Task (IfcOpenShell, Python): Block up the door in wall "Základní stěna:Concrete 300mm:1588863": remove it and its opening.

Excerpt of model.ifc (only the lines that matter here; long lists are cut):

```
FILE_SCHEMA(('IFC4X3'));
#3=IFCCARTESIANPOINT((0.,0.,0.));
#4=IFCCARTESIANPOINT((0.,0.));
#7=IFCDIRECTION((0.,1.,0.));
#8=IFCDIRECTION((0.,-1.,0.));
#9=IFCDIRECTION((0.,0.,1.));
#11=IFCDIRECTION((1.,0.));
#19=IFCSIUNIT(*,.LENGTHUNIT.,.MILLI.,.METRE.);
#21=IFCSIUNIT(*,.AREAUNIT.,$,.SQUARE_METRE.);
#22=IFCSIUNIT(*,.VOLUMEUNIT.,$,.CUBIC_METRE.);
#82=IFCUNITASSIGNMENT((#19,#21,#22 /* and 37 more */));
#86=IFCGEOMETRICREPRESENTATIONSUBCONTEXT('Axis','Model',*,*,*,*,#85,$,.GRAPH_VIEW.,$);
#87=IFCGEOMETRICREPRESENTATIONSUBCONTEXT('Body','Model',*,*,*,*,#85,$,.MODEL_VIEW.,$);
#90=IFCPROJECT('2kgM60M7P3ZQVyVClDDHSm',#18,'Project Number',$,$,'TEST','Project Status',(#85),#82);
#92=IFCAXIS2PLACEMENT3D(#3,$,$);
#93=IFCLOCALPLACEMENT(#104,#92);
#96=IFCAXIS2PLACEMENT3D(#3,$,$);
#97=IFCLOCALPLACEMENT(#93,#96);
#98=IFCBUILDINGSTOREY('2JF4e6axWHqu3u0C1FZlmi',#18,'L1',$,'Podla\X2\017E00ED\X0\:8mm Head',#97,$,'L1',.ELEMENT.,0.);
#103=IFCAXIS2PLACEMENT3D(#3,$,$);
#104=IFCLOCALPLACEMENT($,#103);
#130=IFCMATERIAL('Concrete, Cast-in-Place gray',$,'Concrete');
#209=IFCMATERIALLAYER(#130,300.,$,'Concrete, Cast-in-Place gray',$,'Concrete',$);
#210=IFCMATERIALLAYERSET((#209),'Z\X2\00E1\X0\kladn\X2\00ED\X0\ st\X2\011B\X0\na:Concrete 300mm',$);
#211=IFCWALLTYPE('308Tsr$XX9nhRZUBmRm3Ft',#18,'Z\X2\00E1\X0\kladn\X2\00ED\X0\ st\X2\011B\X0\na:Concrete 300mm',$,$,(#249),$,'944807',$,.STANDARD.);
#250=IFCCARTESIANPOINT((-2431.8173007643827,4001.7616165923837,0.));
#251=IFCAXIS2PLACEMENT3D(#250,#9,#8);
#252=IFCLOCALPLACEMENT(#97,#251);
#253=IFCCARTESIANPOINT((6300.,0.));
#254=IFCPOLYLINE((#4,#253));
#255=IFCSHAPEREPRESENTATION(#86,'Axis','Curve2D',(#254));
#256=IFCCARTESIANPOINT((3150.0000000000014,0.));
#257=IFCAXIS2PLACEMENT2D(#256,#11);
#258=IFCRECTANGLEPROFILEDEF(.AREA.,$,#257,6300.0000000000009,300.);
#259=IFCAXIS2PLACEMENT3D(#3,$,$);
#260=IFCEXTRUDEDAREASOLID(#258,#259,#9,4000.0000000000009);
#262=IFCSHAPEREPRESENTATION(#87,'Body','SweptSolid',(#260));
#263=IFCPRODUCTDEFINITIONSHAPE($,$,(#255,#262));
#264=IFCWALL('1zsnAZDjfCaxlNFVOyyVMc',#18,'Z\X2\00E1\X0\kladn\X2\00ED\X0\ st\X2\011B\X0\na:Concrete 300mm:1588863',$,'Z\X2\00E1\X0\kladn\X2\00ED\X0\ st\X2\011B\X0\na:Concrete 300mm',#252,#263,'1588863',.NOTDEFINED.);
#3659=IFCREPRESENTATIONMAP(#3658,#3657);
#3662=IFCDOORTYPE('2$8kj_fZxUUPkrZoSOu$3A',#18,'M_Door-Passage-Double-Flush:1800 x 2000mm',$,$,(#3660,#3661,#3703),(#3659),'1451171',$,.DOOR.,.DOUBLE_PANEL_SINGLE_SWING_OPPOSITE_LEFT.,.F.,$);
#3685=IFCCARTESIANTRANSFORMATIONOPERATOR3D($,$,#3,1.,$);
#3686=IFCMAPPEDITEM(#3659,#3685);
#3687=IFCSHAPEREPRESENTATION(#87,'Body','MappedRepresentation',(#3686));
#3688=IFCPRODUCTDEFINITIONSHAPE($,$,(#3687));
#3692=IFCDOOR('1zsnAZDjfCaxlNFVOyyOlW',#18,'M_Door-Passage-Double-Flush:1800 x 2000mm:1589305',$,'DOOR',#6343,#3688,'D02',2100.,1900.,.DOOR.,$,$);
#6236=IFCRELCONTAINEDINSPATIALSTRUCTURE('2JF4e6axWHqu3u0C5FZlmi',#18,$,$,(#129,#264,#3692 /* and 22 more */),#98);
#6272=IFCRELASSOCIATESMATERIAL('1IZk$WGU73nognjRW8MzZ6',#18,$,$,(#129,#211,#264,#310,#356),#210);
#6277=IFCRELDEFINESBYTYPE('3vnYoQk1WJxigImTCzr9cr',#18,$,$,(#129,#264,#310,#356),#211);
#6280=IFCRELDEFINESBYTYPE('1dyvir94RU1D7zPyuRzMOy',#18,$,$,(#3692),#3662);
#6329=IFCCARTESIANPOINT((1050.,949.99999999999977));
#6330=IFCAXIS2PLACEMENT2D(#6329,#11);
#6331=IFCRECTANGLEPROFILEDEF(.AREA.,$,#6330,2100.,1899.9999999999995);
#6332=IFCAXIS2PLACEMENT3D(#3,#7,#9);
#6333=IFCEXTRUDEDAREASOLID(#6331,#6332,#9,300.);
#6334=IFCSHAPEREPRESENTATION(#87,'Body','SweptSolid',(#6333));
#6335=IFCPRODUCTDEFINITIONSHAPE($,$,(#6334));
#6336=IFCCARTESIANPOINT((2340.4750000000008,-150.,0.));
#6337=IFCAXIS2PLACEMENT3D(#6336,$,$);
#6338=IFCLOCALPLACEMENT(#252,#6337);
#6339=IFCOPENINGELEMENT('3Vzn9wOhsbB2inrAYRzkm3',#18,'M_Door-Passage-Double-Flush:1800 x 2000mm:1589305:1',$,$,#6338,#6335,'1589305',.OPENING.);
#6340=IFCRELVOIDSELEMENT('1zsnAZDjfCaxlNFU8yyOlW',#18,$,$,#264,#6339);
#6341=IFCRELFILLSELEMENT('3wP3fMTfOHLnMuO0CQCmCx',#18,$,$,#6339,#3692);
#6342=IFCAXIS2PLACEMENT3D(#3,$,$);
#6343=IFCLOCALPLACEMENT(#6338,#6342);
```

```python
import ifcopenshell
import ifcopenshell.api.feature
import ifcopenshell.api.root
import ifcopenshell.geom
import ifcopenshell.util.shape

model = ifcopenshell.open("model.ifc")
settings = ifcopenshell.geom.settings()


def volume(element):
    """Net volume in cubic metres, openings subtracted."""
    shape = ifcopenshell.geom.create_shape(settings, element)
    return ifcopenshell.util.shape.get_volume(shape.geometry)


door = model.by_guid("1zsnAZDjfCaxlNFVOyyOlW")
opening = door.FillsVoids[0].RelatingOpeningElement
wall = opening.VoidsElements[0].RelatingBuildingElement
before = volume(wall)

ifcopenshell.api.root.remove_product(model, product=door)
ifcopenshell.api.feature.remove_feature(model, feature=opening)

after = volume(wall)

print(f"wall volume {before:.3f} -> {after:.3f} m3")

model.write("model_v2.ifc")
```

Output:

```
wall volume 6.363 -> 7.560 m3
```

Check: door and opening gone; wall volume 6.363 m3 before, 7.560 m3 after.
